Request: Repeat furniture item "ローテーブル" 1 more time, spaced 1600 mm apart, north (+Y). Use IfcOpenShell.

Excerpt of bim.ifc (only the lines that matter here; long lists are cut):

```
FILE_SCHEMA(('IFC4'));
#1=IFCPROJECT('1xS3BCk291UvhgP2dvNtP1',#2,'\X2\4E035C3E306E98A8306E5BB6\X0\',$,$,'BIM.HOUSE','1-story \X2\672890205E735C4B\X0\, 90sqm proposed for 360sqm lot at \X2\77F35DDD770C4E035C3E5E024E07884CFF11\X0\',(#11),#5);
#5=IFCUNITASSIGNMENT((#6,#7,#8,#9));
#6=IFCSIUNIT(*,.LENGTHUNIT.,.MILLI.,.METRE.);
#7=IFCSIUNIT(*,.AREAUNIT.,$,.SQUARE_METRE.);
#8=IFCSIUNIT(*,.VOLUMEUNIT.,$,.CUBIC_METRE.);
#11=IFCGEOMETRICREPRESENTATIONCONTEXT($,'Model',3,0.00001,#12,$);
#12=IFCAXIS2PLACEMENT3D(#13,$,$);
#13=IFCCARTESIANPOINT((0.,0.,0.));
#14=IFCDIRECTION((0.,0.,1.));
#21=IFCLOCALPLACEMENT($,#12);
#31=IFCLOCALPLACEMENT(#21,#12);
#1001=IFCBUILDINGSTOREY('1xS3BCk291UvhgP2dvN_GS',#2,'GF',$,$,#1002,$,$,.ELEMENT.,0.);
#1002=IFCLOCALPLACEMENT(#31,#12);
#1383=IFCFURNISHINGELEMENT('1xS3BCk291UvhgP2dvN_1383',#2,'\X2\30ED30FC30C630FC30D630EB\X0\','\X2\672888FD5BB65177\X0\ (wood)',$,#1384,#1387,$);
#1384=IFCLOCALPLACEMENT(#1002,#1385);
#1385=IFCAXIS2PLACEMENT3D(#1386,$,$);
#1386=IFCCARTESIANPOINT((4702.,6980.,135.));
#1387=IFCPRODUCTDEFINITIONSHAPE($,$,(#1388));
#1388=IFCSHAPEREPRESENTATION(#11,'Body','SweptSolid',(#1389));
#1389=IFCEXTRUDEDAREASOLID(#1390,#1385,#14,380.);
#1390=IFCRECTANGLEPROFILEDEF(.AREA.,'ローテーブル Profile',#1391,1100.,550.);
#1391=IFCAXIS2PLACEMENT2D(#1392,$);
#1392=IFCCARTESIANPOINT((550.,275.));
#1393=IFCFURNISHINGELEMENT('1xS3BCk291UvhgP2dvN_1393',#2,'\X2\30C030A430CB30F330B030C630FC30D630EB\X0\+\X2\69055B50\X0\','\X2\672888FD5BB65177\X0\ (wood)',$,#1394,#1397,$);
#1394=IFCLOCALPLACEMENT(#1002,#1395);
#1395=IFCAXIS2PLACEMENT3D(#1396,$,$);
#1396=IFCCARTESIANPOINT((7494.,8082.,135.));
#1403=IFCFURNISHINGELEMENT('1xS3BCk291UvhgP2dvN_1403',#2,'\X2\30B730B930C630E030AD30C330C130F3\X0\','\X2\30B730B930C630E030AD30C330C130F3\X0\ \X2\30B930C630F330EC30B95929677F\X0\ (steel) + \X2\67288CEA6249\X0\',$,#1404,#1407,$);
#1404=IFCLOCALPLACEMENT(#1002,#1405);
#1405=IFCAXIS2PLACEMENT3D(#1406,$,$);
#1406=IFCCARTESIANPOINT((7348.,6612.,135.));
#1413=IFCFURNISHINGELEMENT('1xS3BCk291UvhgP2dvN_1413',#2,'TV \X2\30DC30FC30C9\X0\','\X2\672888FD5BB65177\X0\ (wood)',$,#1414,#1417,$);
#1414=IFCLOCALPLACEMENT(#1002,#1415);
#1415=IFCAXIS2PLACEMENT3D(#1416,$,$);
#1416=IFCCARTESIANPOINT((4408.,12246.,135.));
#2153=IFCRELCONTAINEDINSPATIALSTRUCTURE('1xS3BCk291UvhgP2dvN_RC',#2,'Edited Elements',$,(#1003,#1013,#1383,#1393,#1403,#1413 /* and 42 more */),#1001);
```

```python
import numpy as np
import ifcopenshell
import ifcopenshell.api.geometry
import ifcopenshell.api.root
import ifcopenshell.util.element
import ifcopenshell.util.placement
import ifcopenshell.util.unit

model = ifcopenshell.open("bim.ifc")
unit_scale = ifcopenshell.util.unit.calculate_unit_scale(model)


def reuse_history(source, copy):
    """copy_class also copies each property set's owner history, people and application; keep the originals."""
    for rel in copy.IsDefinedBy:
        if rel.is_a("IfcRelDefinesByProperties") and (history := rel.RelatingPropertyDefinition.OwnerHistory):
            rel.RelatingPropertyDefinition.OwnerHistory = source.OwnerHistory
            ifcopenshell.util.element.remove_deep2(model, history)


source = model.by_guid("1xS3BCk291UvhgP2dvN_1383")
base = ifcopenshell.util.placement.get_local_placement(source.ObjectPlacement)
step = np.array([0.0, 1.0, 0.0]) * 1.6 / unit_scale

for i in range(1, 2):
    copy = ifcopenshell.api.root.copy_class(model, product=source)
    copy.Representation = ifcopenshell.util.element.copy_deep(
        model, source.Representation, exclude=["IfcGeometricRepresentationContext", "IfcRepresentationMap"]
    )
    reuse_history(source, copy)
    matrix = base.copy()
    matrix[:3, 3] += i * step
    print("added at", matrix[:3, 3].round(3) + 0.0)
    ifcopenshell.api.geometry.edit_object_placement(model, product=copy, matrix=matrix, is_si=False)

model.write("bim_v2.ifc")
```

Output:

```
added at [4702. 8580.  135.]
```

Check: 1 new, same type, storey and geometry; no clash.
